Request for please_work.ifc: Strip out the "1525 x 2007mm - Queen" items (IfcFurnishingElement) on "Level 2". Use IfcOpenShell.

First a look at what the model holds.

```python
import ifcopenshell
import ifcopenshell.util.element

model = ifcopenshell.open("please_work.ifc")
print(model.schema)
storey = next(s for s in model.by_type("IfcBuildingStorey") if s.Name == "Level 2")
furniture = [e for e in ifcopenshell.util.element.get_decomposition(storey) if e.is_a("IfcFurnishingElement")]
seen = {}
for e in furniture:
    element_type = ifcopenshell.util.element.get_type(e)
    name = element_type.Name if element_type not in (None, e) else None
    seen[name] = seen.get(name, 0) + 1
for name, count in sorted(seen.items(), key=str):
    print(count, "x", name)
```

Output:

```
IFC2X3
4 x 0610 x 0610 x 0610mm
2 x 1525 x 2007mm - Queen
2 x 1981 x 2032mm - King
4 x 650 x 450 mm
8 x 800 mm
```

```python
import ifcopenshell
import ifcopenshell.api.root
import ifcopenshell.util.element

model = ifcopenshell.open("please_work.ifc")

storey = next(s for s in model.by_type("IfcBuildingStorey") if s.Name == "Level 2")
furniture = [e for e in ifcopenshell.util.element.get_decomposition(storey) if e.is_a("IfcFurnishingElement")]
targets = [e for e in furniture if (t := ifcopenshell.util.element.get_type(e)) not in (None, e) and t.Name == "1525 x 2007mm - Queen"]

for e in targets:
    ifcopenshell.api.root.remove_product(model, product=e)
print(len(targets), "removed")

model.write("please_work_updated.ifc")
```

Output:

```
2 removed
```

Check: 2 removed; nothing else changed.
